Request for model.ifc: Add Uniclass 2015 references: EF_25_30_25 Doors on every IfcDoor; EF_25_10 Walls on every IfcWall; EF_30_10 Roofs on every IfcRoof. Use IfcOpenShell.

First a look at what the model holds.

```python
import ifcopenshell

model = ifcopenshell.open("model.ifc")
print(model.schema)
print("classifications:", [c.Name for c in model.by_type("IfcClassification")])
for ifc_class in ("IfcDoor", "IfcRoof", "IfcStair", "IfcWall", "IfcWindow"):
    print(ifc_class, len(model.by_type(ifc_class)))
```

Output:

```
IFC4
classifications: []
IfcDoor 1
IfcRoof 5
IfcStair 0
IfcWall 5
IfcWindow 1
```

```python
import ifcopenshell
import ifcopenshell.api.classification

model = ifcopenshell.open("model.ifc")

system = ifcopenshell.api.classification.add_classification(model, classification="Uniclass 2015")

codes = {
    "IfcDoor": ("EF_25_30_25", "Doors"),
    "IfcWall": ("EF_25_10", "Walls"),
    "IfcRoof": ("EF_30_10", "Roofs"),
}
for ifc_class, (code, name) in codes.items():
    products = model.by_type(ifc_class)
    ifcopenshell.api.classification.add_reference(
        model, products=products, classification=system, identification=code, name=name
    )
    print(code, len(products))

model.write("model_updated.ifc")
```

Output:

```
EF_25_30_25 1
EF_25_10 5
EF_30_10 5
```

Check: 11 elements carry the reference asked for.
